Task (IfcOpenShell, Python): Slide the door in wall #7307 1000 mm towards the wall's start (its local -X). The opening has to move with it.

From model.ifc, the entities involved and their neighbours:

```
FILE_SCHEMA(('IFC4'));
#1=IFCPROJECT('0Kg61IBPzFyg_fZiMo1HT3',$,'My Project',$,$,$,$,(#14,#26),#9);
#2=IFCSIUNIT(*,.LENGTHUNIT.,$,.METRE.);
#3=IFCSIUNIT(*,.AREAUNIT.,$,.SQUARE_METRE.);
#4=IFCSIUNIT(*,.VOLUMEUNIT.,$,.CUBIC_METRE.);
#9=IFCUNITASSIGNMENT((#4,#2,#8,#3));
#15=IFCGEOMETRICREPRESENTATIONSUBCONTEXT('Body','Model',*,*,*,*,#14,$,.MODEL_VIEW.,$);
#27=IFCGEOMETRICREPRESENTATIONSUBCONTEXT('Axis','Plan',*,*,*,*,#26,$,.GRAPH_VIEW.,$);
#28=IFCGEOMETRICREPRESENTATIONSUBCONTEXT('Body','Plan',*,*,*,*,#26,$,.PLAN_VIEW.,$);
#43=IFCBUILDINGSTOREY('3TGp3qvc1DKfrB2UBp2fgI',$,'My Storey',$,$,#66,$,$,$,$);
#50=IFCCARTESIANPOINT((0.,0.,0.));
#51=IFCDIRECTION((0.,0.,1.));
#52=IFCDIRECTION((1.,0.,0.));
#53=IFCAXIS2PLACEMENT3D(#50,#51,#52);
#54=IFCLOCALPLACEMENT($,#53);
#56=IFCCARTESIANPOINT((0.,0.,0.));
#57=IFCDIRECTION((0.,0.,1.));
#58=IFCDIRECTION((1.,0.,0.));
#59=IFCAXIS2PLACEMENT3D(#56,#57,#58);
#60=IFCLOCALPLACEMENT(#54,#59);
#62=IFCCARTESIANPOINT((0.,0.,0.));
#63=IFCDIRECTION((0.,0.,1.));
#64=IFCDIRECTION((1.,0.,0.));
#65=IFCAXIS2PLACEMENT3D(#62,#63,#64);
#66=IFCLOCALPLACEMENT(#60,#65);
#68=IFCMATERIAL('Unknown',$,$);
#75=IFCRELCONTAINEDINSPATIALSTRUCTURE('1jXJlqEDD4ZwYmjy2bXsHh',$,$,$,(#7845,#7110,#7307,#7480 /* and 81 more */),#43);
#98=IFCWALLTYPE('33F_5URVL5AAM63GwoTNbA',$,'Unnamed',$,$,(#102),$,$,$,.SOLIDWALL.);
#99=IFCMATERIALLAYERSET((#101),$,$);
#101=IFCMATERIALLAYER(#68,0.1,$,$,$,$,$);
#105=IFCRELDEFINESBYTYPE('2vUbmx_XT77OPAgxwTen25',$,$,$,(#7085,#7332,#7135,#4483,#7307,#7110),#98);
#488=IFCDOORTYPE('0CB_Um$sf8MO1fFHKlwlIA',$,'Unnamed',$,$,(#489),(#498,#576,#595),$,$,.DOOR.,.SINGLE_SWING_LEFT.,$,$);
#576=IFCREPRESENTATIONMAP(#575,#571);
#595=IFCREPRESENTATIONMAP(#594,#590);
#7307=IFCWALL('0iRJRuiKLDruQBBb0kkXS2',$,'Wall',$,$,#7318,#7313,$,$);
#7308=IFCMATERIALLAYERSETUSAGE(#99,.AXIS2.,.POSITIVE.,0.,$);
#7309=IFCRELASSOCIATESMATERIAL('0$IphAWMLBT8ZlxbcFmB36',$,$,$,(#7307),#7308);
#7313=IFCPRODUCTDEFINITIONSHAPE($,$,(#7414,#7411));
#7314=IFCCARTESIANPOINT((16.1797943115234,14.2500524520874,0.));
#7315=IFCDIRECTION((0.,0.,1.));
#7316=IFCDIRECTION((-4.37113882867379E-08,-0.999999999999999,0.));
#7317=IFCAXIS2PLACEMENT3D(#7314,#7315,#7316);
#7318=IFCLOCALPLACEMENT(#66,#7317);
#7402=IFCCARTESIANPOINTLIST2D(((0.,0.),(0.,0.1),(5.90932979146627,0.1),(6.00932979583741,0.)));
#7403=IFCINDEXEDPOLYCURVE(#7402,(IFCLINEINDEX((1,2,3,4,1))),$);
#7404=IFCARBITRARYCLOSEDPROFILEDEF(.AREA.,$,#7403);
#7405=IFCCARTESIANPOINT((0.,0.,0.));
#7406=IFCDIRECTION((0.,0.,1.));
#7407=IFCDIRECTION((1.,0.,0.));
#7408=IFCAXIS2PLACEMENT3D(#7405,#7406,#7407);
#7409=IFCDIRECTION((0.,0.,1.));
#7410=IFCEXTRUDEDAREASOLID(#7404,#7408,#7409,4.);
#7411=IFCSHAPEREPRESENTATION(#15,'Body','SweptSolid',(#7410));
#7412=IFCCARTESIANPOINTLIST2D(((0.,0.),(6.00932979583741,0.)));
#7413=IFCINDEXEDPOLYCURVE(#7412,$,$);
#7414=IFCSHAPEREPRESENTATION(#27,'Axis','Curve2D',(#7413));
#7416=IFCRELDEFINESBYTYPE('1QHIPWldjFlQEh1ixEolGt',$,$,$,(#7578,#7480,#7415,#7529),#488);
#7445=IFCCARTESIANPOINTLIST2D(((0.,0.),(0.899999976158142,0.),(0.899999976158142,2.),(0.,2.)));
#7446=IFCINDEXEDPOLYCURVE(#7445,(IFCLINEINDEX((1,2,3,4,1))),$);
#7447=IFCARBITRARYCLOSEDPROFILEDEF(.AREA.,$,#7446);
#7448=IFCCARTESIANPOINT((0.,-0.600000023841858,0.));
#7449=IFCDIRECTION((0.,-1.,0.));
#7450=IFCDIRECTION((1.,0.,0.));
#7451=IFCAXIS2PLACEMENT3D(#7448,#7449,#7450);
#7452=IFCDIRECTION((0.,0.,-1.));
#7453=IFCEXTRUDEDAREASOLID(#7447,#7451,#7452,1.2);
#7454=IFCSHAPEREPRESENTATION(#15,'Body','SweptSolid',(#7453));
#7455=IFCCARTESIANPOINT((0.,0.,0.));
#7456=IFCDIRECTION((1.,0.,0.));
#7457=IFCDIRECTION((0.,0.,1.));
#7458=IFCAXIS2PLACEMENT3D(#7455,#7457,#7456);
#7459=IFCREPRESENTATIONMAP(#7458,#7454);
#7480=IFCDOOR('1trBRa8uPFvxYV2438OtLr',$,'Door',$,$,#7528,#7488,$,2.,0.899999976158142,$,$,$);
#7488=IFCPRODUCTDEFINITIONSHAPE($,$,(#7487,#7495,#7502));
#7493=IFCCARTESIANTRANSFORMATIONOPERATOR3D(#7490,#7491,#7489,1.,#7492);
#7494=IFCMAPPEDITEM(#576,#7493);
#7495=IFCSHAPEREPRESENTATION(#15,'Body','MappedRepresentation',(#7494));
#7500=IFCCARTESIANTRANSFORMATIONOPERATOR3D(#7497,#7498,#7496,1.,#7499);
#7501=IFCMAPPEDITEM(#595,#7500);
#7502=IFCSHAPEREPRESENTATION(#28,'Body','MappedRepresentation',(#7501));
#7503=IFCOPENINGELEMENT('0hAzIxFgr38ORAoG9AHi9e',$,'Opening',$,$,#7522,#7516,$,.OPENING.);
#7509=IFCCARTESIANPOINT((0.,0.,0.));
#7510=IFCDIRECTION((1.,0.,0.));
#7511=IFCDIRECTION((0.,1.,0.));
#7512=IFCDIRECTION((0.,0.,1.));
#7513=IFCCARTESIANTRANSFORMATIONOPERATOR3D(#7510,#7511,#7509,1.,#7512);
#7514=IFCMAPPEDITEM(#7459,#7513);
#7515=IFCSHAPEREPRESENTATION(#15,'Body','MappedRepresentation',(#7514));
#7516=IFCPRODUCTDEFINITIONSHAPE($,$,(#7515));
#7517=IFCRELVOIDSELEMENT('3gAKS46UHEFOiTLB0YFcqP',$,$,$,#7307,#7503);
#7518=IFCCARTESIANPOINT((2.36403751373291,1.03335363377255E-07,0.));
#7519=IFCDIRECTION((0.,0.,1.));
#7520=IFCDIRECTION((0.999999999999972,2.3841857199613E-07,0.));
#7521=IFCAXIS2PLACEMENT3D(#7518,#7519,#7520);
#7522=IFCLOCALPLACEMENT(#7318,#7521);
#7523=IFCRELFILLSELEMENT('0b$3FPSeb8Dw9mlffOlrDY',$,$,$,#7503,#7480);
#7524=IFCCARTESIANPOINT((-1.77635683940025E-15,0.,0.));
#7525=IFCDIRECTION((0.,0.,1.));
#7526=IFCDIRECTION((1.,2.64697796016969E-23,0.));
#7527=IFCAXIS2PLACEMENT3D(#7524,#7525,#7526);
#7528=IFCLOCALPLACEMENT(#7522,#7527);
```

```python
import ifcopenshell
import ifcopenshell.api.geometry
import ifcopenshell.util.placement

model = ifcopenshell.open("model.ifc")

door = model.by_guid("1trBRa8uPFvxYV2438OtLr")
opening = door.FillsVoids[0].RelatingOpeningElement
wall = opening.VoidsElements[0].RelatingBuildingElement

wall_matrix = ifcopenshell.util.placement.get_local_placement(wall.ObjectPlacement)
shift = wall_matrix[:3, 0] * -1.0
before = ifcopenshell.util.placement.get_local_placement(door.ObjectPlacement)[:3, 3].copy()

# The door is placed relative to its opening, so it follows when the opening moves.
matrix = ifcopenshell.util.placement.get_local_placement(opening.ObjectPlacement)
matrix[:3, 3] += shift
ifcopenshell.api.geometry.edit_object_placement(
    model, product=opening, matrix=matrix, is_si=False, should_transform_children=True
)

after = ifcopenshell.util.placement.get_local_placement(door.ObjectPlacement)[:3, 3]
print("door moved by", (after - before).round(3) + 0.0)

model.write("model-out.ifc")
```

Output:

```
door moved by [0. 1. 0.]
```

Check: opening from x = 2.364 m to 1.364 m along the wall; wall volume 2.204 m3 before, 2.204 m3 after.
